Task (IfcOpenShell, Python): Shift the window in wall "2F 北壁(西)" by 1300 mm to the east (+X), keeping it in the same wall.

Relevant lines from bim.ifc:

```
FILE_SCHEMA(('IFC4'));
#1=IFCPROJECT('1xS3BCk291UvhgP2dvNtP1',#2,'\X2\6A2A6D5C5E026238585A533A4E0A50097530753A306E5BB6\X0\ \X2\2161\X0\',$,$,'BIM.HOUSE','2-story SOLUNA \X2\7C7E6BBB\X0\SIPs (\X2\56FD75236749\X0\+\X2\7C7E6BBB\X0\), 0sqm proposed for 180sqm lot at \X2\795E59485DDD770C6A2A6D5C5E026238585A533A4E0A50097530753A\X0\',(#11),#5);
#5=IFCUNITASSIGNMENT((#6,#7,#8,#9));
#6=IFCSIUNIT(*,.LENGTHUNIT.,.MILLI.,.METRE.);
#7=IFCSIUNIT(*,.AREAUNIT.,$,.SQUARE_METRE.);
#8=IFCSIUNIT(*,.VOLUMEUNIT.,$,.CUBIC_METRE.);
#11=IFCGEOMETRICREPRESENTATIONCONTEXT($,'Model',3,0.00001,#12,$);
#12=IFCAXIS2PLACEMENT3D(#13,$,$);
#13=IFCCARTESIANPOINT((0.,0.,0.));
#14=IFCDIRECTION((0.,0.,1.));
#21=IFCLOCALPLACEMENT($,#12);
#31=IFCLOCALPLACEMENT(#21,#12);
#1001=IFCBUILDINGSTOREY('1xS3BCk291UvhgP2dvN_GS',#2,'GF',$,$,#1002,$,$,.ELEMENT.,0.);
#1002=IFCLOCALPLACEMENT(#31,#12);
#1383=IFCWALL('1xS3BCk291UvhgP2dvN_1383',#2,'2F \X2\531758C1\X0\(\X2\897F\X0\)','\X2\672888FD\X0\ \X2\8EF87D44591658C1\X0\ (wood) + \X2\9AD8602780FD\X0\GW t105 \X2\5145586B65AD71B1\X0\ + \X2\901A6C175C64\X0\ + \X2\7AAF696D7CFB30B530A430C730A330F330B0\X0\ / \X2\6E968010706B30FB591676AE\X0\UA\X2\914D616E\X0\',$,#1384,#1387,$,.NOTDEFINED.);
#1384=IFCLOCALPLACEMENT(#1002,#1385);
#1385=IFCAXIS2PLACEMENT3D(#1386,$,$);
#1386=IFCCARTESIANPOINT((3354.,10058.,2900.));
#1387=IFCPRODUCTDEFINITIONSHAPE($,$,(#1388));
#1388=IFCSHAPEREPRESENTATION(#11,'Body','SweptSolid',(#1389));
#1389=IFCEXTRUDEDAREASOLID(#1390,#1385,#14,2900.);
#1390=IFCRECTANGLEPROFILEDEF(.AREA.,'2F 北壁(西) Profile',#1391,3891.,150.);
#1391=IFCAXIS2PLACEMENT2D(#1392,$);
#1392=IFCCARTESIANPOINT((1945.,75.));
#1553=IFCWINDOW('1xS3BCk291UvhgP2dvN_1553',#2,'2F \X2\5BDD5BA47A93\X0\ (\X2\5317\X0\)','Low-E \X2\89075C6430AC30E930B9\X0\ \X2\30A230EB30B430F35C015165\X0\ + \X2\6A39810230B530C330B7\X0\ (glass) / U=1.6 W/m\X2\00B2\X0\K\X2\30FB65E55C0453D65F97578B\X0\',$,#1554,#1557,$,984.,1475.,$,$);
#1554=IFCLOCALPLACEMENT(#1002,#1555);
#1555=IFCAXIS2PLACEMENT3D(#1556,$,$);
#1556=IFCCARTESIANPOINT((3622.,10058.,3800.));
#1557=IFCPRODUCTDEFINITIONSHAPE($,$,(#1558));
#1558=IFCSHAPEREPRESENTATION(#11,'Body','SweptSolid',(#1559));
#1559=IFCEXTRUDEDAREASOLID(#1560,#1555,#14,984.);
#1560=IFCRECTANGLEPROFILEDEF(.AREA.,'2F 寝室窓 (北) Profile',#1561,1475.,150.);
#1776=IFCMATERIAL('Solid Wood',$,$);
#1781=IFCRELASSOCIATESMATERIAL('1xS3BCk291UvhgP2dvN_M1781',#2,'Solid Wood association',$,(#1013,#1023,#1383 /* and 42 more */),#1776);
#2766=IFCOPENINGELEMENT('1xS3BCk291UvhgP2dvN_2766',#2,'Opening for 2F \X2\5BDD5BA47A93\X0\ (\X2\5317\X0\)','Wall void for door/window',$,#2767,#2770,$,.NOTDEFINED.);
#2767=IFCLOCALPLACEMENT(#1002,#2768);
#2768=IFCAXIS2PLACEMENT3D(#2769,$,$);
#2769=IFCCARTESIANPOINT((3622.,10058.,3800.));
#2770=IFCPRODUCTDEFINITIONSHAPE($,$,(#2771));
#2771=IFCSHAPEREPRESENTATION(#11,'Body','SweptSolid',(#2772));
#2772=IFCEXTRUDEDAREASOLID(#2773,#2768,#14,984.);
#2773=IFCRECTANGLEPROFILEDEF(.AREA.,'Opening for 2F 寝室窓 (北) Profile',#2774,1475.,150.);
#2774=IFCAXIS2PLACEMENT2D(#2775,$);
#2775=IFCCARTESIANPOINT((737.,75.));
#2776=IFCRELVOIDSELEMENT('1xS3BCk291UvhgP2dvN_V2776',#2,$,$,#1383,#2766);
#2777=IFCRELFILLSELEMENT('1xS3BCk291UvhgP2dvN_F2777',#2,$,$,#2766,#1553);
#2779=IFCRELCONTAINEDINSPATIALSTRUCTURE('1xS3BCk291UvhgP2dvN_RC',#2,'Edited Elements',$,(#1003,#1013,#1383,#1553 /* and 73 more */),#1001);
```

```python
import ifcopenshell
import ifcopenshell.api.geometry
import ifcopenshell.util.placement

model = ifcopenshell.open("bim.ifc")

window = model.by_id(1553)
opening = window.FillsVoids[0].RelatingOpeningElement
wall = opening.VoidsElements[0].RelatingBuildingElement

wall_matrix = ifcopenshell.util.placement.get_local_placement(wall.ObjectPlacement)
shift = wall_matrix[:3, 0] * 1300.0
before = ifcopenshell.util.placement.get_local_placement(window.ObjectPlacement)[:3, 3].copy()

# The window is not placed relative to its opening, so move both.
for product in (opening, window):
    matrix = ifcopenshell.util.placement.get_local_placement(product.ObjectPlacement)
    matrix[:3, 3] += shift
    ifcopenshell.api.geometry.edit_object_placement(model, product=product, matrix=matrix, is_si=False)

after = ifcopenshell.util.placement.get_local_placement(window.ObjectPlacement)[:3, 3]
print("window moved by", (after - before).round(3) + 0.0)

model.write("bim_updated.ifc")
```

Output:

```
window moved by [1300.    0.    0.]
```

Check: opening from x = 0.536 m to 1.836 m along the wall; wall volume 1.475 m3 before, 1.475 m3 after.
